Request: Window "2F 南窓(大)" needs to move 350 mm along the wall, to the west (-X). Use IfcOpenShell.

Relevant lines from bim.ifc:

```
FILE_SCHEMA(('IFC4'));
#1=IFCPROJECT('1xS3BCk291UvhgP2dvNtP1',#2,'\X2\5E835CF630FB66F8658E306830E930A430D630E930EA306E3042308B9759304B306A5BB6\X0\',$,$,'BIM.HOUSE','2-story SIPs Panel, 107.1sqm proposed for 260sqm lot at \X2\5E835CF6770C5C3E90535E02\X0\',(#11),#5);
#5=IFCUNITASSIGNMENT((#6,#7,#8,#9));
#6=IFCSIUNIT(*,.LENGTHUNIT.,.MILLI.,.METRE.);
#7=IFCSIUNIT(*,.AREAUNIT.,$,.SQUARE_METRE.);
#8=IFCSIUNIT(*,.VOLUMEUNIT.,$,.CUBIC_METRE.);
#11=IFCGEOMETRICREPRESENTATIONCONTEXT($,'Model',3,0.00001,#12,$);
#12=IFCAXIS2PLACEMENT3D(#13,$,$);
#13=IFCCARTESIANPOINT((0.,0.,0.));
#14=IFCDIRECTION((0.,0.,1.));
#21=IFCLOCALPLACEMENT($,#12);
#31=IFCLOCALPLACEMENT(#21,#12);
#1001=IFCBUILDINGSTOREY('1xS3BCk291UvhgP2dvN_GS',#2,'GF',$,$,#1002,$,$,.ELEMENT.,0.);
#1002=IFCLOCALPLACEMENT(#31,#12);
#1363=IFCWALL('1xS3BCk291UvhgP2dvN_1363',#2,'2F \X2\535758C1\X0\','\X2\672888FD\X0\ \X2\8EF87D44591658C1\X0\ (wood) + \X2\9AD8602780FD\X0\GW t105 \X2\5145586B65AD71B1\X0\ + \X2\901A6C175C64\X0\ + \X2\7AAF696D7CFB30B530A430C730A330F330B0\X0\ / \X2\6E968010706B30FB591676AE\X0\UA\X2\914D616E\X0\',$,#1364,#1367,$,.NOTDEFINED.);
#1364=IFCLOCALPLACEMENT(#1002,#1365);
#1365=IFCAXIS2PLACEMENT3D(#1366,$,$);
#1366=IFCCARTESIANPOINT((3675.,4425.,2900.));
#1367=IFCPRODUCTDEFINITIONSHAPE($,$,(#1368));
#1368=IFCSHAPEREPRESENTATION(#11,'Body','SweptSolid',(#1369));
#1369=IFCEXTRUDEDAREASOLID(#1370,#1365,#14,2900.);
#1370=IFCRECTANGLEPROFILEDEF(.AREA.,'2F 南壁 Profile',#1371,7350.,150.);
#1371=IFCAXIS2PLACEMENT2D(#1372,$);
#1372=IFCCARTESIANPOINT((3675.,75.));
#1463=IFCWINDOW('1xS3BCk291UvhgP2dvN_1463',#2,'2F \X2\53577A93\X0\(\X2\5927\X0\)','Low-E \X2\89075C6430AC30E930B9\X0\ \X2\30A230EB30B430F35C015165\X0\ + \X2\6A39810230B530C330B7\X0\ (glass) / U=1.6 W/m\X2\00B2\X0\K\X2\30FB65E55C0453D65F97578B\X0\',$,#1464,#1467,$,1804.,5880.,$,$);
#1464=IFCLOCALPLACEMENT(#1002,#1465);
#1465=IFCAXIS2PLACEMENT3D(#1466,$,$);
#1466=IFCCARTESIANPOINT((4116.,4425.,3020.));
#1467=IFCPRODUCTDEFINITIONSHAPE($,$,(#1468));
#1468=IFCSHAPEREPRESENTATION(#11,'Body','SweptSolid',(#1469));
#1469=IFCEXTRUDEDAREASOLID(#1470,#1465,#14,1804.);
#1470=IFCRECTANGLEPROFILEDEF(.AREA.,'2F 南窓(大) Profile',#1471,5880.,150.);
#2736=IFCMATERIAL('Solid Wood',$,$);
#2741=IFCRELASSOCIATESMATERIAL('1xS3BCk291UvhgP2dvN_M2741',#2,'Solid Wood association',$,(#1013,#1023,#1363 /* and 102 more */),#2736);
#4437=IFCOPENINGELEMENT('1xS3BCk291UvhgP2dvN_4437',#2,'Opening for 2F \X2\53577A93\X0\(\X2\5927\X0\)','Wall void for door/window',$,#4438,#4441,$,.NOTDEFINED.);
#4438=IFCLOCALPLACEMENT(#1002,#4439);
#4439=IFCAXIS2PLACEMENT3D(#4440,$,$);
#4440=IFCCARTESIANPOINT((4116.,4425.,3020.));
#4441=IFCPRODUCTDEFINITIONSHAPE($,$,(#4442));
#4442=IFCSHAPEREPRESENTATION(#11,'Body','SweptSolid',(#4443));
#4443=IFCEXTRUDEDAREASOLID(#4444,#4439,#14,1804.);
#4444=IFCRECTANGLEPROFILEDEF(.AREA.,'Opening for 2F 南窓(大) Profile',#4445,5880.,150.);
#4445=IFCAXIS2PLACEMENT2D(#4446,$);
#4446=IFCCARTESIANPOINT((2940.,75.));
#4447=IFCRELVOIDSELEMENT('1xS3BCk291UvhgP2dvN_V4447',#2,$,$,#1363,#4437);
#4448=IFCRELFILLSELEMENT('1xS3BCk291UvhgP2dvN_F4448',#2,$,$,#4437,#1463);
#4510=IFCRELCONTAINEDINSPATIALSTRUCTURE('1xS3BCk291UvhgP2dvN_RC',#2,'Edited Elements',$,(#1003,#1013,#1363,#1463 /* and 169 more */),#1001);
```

```python
import ifcopenshell
import ifcopenshell.api.geometry
import ifcopenshell.util.placement
import ifcopenshell.util.unit

model = ifcopenshell.open("bim.ifc")
unit_scale = ifcopenshell.util.unit.calculate_unit_scale(model)

window = model.by_guid("1xS3BCk291UvhgP2dvN_1463")
opening = window.FillsVoids[0].RelatingOpeningElement
wall = opening.VoidsElements[0].RelatingBuildingElement

wall_matrix = ifcopenshell.util.placement.get_local_placement(wall.ObjectPlacement)
shift = wall_matrix[:3, 0] * -0.35 / unit_scale
before = ifcopenshell.util.placement.get_local_placement(window.ObjectPlacement)[:3, 3].copy()

# The window is not placed relative to its opening, so move both.
for product in (opening, window):
    matrix = ifcopenshell.util.placement.get_local_placement(product.ObjectPlacement)
    matrix[:3, 3] += shift
    ifcopenshell.api.geometry.edit_object_placement(model, product=product, matrix=matrix, is_si=False)

after = ifcopenshell.util.placement.get_local_placement(window.ObjectPlacement)[:3, 3]
print("window moved by", (after - before).round(3) + 0.0)

model.write("bim_v2.ifc")
```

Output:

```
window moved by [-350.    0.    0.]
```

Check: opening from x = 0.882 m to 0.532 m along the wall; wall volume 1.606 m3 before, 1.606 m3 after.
